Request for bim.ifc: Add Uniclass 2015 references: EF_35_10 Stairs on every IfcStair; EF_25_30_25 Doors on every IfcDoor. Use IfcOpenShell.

First a look at what the model holds.

```python
import ifcopenshell

model = ifcopenshell.open("bim.ifc")
print(model.schema)
print("classifications:", [c.Name for c in model.by_type("IfcClassification")])
for ifc_class in ("IfcDoor", "IfcRoof", "IfcStair", "IfcWall", "IfcWindow"):
    print(ifc_class, len(model.by_type(ifc_class)))
```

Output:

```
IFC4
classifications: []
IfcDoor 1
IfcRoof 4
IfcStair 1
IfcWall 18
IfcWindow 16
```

```python
import ifcopenshell
import ifcopenshell.api.classification

model = ifcopenshell.open("bim.ifc")

system = ifcopenshell.api.classification.add_classification(model, classification="Uniclass 2015")

codes = {
    "IfcStair": ("EF_35_10", "Stairs"),
    "IfcDoor": ("EF_25_30_25", "Doors"),
}
for ifc_class, (code, name) in codes.items():
    products = model.by_type(ifc_class)
    ifcopenshell.api.classification.add_reference(
        model, products=products, classification=system, identification=code, name=name
    )
    print(code, len(products))

model.write("bim_rev.ifc")
```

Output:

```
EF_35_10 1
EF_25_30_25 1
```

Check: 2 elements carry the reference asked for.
